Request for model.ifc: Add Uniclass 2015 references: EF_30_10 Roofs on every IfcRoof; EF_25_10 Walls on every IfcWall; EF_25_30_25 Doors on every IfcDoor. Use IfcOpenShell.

First a look at what the model holds.

```python
import ifcopenshell

model = ifcopenshell.open("model.ifc")
print(model.schema)
print("classifications:", [c.Name for c in model.by_type("IfcClassification")])
for ifc_class in ("IfcDoor", "IfcRoof", "IfcStair", "IfcWall", "IfcWindow"):
    print(ifc_class, len(model.by_type(ifc_class)))
```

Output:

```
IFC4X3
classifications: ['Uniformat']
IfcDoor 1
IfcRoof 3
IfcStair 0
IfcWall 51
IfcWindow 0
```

```python
import ifcopenshell
import ifcopenshell.api.classification

model = ifcopenshell.open("model.ifc")

system = ifcopenshell.api.classification.add_classification(model, classification="Uniclass 2015")

codes = {
    "IfcRoof": ("EF_30_10", "Roofs"),
    "IfcWall": ("EF_25_10", "Walls"),
    "IfcDoor": ("EF_25_30_25", "Doors"),
}
for ifc_class, (code, name) in codes.items():
    products = model.by_type(ifc_class)
    ifcopenshell.api.classification.add_reference(
        model, products=products, classification=system, identification=code, name=name
    )
    print(code, len(products))

model.write("model_edited.ifc")
```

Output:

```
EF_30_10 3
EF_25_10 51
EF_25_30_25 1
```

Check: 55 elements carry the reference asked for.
